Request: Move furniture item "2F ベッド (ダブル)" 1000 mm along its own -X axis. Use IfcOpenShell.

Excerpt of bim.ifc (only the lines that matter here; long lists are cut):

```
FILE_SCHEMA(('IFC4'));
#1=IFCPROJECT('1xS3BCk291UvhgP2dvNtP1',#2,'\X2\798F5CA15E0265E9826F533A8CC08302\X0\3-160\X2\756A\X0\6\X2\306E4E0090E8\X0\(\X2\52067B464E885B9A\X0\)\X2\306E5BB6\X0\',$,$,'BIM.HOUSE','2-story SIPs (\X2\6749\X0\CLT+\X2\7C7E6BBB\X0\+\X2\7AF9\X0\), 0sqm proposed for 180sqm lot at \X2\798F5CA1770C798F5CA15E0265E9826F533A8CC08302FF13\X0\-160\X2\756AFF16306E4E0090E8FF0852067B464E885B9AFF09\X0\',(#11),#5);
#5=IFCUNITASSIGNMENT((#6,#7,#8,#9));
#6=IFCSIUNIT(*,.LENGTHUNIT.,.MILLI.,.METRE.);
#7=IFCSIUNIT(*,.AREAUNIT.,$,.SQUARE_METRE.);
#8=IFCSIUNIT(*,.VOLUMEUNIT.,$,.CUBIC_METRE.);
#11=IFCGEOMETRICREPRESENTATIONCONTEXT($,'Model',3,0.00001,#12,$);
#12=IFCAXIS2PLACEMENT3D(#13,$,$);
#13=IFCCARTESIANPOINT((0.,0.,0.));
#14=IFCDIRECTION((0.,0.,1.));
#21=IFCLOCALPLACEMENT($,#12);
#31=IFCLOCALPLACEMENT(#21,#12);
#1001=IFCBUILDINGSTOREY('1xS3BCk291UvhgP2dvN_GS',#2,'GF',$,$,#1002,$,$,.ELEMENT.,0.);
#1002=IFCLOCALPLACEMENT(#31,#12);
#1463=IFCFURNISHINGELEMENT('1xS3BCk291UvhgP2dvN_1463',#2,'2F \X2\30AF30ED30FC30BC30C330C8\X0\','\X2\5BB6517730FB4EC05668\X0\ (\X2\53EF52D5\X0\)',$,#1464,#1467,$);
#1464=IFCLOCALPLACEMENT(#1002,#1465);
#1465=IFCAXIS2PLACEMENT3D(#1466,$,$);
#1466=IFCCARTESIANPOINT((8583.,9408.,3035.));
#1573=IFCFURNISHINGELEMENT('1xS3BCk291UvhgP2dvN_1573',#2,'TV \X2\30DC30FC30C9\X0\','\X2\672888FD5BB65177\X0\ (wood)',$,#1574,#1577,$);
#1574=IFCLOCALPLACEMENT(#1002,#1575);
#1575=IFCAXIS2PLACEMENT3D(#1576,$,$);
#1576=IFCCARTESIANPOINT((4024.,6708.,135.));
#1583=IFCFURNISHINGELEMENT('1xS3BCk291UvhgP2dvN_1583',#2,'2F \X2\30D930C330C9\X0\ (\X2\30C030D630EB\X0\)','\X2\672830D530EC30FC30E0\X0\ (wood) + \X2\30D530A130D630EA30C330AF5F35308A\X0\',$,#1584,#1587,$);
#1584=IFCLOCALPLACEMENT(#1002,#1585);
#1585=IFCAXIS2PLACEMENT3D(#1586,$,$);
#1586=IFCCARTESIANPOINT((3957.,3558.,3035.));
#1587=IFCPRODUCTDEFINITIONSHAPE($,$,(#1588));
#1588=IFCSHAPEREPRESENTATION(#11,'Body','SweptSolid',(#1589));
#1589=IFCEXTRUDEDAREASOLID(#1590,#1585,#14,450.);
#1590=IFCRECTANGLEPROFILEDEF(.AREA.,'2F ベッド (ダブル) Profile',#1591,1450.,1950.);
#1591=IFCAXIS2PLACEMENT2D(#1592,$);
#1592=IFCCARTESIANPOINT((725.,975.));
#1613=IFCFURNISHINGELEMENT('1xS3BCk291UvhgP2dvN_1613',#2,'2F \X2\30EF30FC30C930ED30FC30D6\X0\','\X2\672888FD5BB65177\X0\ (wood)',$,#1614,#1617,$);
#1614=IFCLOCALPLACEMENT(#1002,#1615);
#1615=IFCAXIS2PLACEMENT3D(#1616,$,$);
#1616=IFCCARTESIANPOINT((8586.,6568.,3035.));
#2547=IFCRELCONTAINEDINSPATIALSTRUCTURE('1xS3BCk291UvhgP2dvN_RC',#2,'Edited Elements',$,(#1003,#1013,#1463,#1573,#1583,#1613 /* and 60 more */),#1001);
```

```python
import ifcopenshell
import ifcopenshell.api.geometry
import ifcopenshell.util.placement
import ifcopenshell.util.unit

model = ifcopenshell.open("bim.ifc")
unit_scale = ifcopenshell.util.unit.calculate_unit_scale(model)

item = model.by_guid("1xS3BCk291UvhgP2dvN_1583")
matrix = ifcopenshell.util.placement.get_local_placement(item.ObjectPlacement)
matrix[:3, 3] -= matrix[:3, 0] * 1 / unit_scale
ifcopenshell.api.geometry.edit_object_placement(model, product=item, matrix=matrix, is_si=False)

print(ifcopenshell.util.placement.get_local_placement(item.ObjectPlacement).round(3) + 0.0)

model.write("bim_rev.ifc")
```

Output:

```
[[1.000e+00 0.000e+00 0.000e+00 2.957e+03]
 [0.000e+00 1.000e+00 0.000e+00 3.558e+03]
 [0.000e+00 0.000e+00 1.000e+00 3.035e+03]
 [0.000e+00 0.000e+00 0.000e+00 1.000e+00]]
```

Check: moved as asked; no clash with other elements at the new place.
